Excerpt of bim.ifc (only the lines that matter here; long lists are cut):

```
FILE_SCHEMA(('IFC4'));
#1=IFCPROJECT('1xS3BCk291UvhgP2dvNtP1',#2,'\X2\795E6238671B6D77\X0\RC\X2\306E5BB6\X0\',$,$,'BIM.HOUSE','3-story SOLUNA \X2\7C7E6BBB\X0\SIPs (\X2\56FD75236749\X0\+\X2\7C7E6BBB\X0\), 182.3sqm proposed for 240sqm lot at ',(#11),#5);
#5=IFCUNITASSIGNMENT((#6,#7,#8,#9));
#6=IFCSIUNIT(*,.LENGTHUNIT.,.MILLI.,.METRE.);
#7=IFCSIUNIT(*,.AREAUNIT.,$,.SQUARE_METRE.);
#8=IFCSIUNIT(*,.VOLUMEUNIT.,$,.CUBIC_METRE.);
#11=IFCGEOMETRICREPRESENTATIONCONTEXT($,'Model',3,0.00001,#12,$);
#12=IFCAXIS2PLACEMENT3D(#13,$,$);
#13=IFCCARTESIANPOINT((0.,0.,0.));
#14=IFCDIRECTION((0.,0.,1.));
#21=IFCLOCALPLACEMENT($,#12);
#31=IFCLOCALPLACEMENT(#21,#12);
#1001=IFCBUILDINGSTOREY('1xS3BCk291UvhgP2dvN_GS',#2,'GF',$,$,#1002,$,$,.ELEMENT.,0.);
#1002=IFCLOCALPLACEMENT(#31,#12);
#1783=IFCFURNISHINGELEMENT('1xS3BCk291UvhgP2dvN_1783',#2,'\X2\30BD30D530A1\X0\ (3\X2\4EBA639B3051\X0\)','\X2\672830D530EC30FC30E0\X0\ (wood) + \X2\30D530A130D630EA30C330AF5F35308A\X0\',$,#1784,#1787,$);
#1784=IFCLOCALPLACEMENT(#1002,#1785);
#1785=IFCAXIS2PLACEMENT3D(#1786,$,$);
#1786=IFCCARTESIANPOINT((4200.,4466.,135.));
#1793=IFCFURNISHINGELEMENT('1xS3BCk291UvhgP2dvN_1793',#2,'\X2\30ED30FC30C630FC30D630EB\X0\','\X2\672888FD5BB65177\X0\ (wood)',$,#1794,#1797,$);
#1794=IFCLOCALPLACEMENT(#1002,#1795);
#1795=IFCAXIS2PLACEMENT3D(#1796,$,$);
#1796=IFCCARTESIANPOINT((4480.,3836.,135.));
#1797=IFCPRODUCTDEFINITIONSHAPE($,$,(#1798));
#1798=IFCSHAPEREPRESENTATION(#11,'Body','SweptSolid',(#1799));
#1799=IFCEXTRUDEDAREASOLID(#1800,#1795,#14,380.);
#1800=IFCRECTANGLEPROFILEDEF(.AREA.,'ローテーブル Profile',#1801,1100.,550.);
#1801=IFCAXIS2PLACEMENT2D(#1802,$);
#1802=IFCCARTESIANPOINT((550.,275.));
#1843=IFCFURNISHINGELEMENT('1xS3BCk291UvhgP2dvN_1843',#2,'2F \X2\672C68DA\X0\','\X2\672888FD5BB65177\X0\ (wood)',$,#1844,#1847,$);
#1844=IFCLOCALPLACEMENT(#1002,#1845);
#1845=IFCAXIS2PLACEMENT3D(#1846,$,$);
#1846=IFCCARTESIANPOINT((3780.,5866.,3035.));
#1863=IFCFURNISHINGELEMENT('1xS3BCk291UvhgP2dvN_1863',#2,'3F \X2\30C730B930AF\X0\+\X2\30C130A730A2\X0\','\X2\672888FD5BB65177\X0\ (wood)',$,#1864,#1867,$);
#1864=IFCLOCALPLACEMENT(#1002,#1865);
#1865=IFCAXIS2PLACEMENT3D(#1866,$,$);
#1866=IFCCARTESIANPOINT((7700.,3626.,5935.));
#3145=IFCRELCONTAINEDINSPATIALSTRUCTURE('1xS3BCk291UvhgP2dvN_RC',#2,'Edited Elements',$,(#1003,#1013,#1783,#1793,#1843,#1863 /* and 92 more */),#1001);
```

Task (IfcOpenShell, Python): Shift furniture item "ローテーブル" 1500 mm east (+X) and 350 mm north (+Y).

```python
import ifcopenshell
import ifcopenshell.api.geometry
import ifcopenshell.util.placement

model = ifcopenshell.open("bim.ifc")

item = model.by_guid("1xS3BCk291UvhgP2dvN_1793")
matrix = ifcopenshell.util.placement.get_local_placement(item.ObjectPlacement)
matrix[0, 3] += 1500.0
matrix[1, 3] += 350.0
ifcopenshell.api.geometry.edit_object_placement(model, product=item, matrix=matrix, is_si=False)

print(ifcopenshell.util.placement.get_local_placement(item.ObjectPlacement).round(3) + 0.0)

model.write("bim_updated.ifc")
```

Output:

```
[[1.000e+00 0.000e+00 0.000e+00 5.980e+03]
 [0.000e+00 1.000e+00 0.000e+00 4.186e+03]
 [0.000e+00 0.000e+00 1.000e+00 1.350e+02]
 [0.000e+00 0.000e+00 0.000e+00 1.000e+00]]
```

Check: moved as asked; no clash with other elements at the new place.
